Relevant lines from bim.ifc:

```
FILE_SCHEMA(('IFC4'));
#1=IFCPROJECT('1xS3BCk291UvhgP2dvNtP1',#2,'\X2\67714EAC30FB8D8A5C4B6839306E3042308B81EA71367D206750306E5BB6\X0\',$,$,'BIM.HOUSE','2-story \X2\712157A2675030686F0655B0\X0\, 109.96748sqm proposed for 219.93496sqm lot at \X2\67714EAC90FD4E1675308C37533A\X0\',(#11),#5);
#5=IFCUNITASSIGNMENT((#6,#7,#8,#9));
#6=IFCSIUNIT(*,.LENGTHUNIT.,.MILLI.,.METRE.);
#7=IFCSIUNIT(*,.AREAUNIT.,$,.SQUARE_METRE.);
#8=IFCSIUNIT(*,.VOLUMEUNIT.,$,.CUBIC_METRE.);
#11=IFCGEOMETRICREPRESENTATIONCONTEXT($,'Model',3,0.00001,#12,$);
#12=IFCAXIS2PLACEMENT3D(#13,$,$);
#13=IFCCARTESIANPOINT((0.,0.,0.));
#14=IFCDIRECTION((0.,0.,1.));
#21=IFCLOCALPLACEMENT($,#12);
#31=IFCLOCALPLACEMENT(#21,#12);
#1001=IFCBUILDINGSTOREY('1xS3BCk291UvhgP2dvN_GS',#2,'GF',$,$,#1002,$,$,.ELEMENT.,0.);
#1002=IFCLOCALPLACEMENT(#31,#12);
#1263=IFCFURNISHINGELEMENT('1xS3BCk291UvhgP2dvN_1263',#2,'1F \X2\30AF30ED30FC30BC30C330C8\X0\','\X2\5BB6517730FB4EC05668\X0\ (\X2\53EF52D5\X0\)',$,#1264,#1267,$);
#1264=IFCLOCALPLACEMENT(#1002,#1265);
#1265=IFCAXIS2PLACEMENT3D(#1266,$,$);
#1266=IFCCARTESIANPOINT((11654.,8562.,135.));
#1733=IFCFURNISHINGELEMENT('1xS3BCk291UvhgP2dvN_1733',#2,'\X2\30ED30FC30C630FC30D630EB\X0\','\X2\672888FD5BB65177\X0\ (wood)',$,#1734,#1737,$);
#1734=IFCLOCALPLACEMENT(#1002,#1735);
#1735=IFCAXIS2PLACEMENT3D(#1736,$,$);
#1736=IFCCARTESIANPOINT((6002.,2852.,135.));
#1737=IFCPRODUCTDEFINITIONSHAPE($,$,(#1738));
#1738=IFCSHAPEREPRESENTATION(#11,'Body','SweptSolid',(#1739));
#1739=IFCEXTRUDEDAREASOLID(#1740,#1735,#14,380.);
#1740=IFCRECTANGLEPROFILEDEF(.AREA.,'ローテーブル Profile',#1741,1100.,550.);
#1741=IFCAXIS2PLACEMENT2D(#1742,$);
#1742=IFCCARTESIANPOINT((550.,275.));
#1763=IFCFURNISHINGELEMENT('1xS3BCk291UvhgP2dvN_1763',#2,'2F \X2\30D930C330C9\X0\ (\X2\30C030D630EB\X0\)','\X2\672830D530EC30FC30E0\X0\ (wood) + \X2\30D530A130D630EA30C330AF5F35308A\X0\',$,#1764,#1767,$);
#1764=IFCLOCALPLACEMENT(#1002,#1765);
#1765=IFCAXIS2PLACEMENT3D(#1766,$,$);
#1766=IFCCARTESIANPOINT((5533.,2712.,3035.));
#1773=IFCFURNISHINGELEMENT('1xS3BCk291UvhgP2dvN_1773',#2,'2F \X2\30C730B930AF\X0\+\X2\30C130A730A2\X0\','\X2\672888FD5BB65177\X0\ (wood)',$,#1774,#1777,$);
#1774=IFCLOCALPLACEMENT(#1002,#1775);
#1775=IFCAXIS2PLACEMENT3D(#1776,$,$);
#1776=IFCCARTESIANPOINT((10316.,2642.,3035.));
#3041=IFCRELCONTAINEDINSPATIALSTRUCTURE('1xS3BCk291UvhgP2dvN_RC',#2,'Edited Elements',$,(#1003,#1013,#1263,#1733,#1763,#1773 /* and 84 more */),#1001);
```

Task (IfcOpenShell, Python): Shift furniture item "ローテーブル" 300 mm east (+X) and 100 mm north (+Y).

```python
import ifcopenshell
import ifcopenshell.api.geometry
import ifcopenshell.util.placement
import ifcopenshell.util.unit

model = ifcopenshell.open("bim.ifc")
unit_scale = ifcopenshell.util.unit.calculate_unit_scale(model)

item = model.by_id(1733)
matrix = ifcopenshell.util.placement.get_local_placement(item.ObjectPlacement)
matrix[0, 3] += 0.3 / unit_scale
matrix[1, 3] += 0.1 / unit_scale
ifcopenshell.api.geometry.edit_object_placement(model, product=item, matrix=matrix, is_si=False)

print(ifcopenshell.util.placement.get_local_placement(item.ObjectPlacement).round(3) + 0.0)

model.write("bim_rev.ifc")
```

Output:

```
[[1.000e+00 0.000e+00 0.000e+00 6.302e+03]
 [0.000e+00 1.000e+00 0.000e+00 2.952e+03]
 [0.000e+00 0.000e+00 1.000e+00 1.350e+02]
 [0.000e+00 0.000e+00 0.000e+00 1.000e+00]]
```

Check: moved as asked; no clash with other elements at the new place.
